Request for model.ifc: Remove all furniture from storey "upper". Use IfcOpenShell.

First a look at what the model holds.

```python
import ifcopenshell
import ifcopenshell.util.element

model = ifcopenshell.open("model.ifc")
print(model.schema)
storey = next(s for s in model.by_type("IfcBuildingStorey") if s.Name == "upper")
furniture = [e for e in ifcopenshell.util.element.get_decomposition(storey) if e.is_a("IfcFurnishingElement")]
seen = {}
for e in furniture:
    element_type = ifcopenshell.util.element.get_type(e)
    name = element_type.Name if element_type not in (None, e) else None
    seen[name] = seen.get(name, 0) + 1
for name, count in sorted(seen.items(), key=str):
    print(count, "x", name)
```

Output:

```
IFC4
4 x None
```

```python
import ifcopenshell
import ifcopenshell.api.root
import ifcopenshell.util.element

model = ifcopenshell.open("model.ifc")

storey = next(s for s in model.by_type("IfcBuildingStorey") if s.Name == "upper")
furniture = [e for e in ifcopenshell.util.element.get_decomposition(storey) if e.is_a("IfcFurnishingElement")]

for e in furniture:
    ifcopenshell.api.root.remove_product(model, product=e)
print(len(furniture), "removed")

model.write("model_v2.ifc")
```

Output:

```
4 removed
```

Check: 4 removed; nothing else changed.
